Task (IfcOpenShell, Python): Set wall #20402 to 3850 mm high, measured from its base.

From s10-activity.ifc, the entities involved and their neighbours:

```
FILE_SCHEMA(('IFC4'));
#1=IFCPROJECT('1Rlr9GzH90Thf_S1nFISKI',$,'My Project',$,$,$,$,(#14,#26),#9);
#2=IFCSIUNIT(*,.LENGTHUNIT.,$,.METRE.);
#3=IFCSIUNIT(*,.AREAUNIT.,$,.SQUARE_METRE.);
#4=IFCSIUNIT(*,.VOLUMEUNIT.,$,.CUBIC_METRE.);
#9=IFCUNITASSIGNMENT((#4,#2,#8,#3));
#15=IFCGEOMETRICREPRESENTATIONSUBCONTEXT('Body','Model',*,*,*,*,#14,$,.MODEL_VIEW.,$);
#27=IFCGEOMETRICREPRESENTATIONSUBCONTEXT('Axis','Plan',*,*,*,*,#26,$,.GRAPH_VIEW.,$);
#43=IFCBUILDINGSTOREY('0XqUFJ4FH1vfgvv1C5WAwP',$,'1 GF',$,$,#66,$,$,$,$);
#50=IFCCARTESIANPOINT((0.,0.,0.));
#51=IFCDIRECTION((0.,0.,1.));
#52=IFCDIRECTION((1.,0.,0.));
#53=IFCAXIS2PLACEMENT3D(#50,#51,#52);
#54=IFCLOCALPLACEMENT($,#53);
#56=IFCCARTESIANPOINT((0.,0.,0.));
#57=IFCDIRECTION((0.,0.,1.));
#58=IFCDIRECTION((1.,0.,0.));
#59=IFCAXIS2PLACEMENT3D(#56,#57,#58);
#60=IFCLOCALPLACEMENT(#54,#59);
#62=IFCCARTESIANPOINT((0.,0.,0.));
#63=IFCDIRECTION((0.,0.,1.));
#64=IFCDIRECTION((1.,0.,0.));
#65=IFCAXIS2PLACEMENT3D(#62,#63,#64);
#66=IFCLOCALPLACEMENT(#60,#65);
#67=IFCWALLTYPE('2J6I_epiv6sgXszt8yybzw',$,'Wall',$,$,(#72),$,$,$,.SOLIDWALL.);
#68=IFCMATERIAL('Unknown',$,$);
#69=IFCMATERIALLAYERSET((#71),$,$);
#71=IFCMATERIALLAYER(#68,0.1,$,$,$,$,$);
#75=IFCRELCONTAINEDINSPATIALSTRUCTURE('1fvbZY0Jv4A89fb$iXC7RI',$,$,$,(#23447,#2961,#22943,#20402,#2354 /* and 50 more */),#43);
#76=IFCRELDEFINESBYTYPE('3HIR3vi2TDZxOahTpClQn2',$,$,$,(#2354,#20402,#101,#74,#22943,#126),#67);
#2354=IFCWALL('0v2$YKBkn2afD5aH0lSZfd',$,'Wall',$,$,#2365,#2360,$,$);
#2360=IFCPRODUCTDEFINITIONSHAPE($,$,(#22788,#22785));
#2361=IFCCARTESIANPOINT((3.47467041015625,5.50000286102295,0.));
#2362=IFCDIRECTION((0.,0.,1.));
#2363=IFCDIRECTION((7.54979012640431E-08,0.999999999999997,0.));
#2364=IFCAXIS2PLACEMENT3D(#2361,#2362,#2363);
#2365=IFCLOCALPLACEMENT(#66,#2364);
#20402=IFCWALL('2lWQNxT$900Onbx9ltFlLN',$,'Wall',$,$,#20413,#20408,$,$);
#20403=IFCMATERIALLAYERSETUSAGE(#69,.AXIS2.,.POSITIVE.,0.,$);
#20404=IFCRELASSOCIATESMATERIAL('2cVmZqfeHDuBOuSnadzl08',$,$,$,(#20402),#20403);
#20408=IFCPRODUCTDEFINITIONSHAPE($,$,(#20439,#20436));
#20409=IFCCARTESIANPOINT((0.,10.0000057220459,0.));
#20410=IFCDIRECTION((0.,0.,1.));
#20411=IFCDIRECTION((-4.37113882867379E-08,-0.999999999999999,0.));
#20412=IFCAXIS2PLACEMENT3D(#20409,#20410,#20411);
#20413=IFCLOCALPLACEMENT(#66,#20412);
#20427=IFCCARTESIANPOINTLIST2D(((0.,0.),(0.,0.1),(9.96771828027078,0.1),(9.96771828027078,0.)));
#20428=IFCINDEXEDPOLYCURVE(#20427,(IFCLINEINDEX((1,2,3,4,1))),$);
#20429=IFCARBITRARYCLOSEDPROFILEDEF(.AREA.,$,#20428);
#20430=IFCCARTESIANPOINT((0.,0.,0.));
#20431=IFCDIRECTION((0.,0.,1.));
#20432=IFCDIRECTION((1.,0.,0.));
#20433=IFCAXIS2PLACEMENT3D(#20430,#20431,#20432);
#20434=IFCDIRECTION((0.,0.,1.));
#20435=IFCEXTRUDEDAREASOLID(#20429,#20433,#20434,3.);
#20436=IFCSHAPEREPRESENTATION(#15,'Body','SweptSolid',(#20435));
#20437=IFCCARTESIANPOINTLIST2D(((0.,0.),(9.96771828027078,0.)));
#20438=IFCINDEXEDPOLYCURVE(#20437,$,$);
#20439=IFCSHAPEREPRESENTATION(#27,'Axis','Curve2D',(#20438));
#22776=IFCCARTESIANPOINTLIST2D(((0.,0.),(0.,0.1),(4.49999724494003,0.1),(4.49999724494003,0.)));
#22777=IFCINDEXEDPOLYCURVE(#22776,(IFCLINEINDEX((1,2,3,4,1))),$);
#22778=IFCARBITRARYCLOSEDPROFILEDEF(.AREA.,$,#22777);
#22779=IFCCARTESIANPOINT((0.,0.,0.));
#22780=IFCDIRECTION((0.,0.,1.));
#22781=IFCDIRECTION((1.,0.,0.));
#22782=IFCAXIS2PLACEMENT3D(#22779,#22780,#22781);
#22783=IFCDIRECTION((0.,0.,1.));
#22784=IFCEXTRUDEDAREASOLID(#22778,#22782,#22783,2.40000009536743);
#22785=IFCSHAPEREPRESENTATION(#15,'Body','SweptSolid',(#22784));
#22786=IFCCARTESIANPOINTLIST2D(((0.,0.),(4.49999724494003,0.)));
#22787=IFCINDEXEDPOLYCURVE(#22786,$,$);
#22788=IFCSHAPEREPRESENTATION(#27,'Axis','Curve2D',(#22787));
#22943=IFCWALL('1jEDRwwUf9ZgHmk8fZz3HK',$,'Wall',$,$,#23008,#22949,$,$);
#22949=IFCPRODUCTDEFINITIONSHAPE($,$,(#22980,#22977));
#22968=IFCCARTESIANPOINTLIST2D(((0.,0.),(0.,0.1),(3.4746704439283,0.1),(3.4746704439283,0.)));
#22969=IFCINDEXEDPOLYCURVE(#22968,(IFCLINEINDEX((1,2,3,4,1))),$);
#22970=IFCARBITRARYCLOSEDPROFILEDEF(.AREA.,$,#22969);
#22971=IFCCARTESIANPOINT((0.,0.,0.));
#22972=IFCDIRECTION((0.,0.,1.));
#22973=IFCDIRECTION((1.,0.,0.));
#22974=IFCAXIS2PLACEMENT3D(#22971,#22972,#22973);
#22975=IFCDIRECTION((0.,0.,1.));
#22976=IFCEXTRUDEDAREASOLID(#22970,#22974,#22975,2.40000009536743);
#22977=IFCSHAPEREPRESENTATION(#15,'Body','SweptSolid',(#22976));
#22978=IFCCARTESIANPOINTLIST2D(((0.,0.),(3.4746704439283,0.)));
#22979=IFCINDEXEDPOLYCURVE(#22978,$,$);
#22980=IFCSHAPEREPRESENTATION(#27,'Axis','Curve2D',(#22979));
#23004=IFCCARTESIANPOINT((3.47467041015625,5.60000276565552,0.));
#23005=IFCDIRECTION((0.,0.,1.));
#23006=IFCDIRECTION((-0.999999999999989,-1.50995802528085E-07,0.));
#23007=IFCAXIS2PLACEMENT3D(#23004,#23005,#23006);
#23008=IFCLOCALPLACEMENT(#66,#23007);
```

```python
import ifcopenshell
import ifcopenshell.geom
import ifcopenshell.util.representation
import ifcopenshell.util.shape

model = ifcopenshell.open("s10-activity.ifc")
settings = ifcopenshell.geom.settings()


def volume(element):
    """Net volume in cubic metres, openings subtracted."""
    shape = ifcopenshell.geom.create_shape(settings, element)
    return ifcopenshell.util.shape.get_volume(shape.geometry)


wall = model.by_guid("2lWQNxT$900Onbx9ltFlLN")
before = volume(wall)

body = ifcopenshell.util.representation.get_representation(wall, "Model", "Body")
solid = body.Items[0]
old_height = solid.Depth
solid.Depth = 3.85
after = volume(wall)

print(f"height {old_height:g} -> {solid.Depth:g}, volume {before:.3f} -> {after:.3f} m3")

model.write("s10-activity-out.ifc")
```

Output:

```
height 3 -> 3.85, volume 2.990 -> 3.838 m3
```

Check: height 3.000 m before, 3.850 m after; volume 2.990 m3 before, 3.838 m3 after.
